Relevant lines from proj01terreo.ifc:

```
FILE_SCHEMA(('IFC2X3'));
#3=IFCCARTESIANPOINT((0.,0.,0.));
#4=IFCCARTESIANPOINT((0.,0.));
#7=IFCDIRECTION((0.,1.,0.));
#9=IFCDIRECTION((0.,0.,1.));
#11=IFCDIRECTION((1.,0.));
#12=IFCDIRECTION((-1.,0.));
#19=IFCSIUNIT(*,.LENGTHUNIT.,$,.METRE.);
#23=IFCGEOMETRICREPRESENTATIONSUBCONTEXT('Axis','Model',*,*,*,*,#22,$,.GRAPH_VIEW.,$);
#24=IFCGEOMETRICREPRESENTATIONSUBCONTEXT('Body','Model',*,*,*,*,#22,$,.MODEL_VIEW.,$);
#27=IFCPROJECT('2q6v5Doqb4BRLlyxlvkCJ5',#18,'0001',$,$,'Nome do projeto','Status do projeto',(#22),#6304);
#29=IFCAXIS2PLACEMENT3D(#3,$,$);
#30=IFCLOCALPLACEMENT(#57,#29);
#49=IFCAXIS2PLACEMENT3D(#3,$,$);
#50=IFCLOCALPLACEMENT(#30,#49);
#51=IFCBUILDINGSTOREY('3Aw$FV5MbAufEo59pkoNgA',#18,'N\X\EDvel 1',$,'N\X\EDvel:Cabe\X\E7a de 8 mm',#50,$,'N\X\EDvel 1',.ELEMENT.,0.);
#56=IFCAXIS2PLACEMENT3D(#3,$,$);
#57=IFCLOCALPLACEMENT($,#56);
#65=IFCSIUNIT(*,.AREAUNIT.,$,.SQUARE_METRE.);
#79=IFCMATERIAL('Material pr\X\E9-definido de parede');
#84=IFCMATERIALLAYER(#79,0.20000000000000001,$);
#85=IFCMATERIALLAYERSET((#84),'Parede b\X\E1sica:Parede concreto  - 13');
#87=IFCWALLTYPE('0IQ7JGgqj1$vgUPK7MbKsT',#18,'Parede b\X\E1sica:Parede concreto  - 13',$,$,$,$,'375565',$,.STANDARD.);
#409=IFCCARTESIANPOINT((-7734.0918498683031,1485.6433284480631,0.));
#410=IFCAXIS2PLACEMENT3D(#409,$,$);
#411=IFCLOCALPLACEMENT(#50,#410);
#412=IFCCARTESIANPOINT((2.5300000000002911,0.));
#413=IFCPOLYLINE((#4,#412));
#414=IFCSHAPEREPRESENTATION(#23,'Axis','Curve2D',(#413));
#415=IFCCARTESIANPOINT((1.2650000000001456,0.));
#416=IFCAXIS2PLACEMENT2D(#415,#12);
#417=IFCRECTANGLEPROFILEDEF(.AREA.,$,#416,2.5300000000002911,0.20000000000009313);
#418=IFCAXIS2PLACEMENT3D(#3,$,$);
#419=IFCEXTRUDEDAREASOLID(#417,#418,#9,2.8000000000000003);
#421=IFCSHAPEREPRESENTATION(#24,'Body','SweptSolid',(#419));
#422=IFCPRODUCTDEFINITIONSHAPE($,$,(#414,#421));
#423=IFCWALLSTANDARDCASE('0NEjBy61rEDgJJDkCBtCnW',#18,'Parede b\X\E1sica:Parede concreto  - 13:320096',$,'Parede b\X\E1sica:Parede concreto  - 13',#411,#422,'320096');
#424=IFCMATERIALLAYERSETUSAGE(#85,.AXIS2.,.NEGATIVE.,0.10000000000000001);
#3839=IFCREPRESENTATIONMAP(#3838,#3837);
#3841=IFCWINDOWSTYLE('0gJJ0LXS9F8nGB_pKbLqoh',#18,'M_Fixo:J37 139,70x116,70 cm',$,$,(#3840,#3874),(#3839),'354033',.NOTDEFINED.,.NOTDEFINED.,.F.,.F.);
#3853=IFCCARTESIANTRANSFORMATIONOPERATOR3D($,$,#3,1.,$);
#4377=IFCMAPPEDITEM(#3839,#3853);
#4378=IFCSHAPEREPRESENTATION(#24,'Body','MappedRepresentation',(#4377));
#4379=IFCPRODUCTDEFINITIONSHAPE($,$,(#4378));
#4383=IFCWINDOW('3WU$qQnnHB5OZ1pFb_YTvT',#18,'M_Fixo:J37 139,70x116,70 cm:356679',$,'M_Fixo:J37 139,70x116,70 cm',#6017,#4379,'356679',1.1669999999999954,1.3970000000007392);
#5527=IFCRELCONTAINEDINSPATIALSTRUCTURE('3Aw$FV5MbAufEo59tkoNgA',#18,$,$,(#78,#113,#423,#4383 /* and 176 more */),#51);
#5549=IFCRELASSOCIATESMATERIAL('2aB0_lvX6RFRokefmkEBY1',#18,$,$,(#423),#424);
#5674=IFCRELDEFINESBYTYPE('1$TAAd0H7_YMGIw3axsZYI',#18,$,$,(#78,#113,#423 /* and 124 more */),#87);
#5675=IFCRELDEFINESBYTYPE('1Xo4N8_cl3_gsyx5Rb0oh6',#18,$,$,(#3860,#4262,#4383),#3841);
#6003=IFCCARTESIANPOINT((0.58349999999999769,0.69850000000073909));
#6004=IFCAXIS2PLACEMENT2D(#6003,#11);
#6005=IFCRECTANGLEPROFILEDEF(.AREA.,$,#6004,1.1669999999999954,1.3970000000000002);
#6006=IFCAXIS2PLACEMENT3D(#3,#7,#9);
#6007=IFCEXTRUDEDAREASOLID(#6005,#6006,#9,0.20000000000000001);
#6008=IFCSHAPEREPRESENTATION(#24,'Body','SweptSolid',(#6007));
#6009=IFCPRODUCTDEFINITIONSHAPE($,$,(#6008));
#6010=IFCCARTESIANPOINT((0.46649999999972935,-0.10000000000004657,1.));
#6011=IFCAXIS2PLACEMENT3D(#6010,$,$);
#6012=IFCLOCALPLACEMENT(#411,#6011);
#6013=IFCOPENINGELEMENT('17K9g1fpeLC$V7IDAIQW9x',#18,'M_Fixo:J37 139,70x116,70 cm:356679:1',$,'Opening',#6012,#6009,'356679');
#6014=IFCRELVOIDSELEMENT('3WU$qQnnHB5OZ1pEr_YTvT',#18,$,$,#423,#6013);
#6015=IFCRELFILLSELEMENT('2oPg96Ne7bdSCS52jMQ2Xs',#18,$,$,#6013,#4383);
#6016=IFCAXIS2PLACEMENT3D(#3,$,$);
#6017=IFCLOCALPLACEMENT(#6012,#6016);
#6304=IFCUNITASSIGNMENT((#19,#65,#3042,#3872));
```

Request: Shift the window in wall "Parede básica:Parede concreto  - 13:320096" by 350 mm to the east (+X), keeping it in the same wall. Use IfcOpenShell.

```python
import ifcopenshell
import ifcopenshell.api.geometry
import ifcopenshell.util.placement
import ifcopenshell.util.unit

model = ifcopenshell.open("proj01terreo.ifc")
unit_scale = ifcopenshell.util.unit.calculate_unit_scale(model)

window = model.by_id(4383)
opening = window.FillsVoids[0].RelatingOpeningElement
wall = opening.VoidsElements[0].RelatingBuildingElement

wall_matrix = ifcopenshell.util.placement.get_local_placement(wall.ObjectPlacement)
shift = wall_matrix[:3, 0] * 0.35 / unit_scale
before = ifcopenshell.util.placement.get_local_placement(window.ObjectPlacement)[:3, 3].copy()

# The window is placed relative to its opening, so it follows when the opening moves.
matrix = ifcopenshell.util.placement.get_local_placement(opening.ObjectPlacement)
matrix[:3, 3] += shift
ifcopenshell.api.geometry.edit_object_placement(
    model, product=opening, matrix=matrix, is_si=False, should_transform_children=True
)

after = ifcopenshell.util.placement.get_local_placement(window.ObjectPlacement)[:3, 3]
print("window moved by", (after - before).round(3) + 0.0)

model.write("proj01terreo_v2.ifc")
```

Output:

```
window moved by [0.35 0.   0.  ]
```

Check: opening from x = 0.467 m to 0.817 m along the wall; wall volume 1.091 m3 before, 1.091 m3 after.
